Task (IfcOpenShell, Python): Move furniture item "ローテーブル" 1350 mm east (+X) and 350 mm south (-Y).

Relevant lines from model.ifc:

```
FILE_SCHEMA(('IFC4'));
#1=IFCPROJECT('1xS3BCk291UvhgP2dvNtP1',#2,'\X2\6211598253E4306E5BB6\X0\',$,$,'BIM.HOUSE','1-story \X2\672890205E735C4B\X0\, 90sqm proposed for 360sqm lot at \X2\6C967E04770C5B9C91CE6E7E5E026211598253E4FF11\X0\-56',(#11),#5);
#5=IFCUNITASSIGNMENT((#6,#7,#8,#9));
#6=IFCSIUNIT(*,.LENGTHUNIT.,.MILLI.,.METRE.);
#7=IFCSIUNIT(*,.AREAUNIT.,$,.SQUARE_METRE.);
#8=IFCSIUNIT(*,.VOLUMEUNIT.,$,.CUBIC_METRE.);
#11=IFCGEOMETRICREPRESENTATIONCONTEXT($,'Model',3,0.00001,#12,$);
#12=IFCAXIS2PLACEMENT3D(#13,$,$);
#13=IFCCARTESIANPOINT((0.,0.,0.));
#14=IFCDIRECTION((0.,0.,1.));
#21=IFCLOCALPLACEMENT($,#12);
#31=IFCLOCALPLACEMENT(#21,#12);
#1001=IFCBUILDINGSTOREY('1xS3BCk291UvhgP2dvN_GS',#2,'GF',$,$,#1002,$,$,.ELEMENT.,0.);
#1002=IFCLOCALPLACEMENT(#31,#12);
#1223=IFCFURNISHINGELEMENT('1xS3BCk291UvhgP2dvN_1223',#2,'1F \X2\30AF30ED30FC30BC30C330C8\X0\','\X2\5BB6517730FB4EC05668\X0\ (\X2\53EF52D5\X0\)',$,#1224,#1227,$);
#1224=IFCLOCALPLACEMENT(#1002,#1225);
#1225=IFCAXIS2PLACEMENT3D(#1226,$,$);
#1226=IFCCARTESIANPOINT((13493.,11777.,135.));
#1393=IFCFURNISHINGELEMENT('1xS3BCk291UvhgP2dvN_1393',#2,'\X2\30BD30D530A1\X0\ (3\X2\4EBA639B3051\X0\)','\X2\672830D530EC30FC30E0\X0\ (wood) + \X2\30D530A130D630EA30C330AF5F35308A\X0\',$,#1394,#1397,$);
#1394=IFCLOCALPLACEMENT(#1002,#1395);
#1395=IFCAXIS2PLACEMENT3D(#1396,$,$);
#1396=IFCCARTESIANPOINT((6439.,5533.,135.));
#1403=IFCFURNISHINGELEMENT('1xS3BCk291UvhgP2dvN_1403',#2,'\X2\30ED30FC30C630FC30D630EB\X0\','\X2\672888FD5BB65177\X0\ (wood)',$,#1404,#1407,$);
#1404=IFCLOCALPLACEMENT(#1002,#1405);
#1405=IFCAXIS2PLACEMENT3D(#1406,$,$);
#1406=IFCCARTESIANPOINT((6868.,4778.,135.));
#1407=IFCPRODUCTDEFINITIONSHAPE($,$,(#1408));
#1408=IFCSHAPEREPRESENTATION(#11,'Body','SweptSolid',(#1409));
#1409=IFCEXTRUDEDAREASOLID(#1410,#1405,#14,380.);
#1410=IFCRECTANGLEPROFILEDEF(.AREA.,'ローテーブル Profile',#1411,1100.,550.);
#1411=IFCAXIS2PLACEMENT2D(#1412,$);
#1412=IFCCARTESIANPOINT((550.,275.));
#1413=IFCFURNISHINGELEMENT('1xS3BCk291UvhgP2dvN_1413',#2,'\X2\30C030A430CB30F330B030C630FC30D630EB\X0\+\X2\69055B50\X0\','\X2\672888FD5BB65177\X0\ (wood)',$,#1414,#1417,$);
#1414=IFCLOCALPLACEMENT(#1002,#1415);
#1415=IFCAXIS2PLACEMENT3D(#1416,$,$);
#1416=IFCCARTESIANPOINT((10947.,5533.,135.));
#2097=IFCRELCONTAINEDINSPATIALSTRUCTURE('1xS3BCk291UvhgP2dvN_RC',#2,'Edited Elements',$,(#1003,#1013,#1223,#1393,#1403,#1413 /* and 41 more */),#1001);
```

```python
import ifcopenshell
import ifcopenshell.api.geometry
import ifcopenshell.util.placement
import ifcopenshell.util.unit

model = ifcopenshell.open("model.ifc")
unit_scale = ifcopenshell.util.unit.calculate_unit_scale(model)

item = model.by_guid("1xS3BCk291UvhgP2dvN_1403")
matrix = ifcopenshell.util.placement.get_local_placement(item.ObjectPlacement)
matrix[0, 3] += 1.35 / unit_scale
matrix[1, 3] -= 0.35 / unit_scale
ifcopenshell.api.geometry.edit_object_placement(model, product=item, matrix=matrix, is_si=False)

print(ifcopenshell.util.placement.get_local_placement(item.ObjectPlacement).round(3) + 0.0)

model.write("model_rev.ifc")
```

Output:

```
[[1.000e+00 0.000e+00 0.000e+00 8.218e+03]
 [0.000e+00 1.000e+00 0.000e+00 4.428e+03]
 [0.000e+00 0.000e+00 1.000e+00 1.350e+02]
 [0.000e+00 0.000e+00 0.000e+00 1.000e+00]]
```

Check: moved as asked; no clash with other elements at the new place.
